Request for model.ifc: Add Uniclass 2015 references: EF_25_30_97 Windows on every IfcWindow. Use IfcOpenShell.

First a look at what the model holds.

```python
import ifcopenshell

model = ifcopenshell.open("model.ifc")
print(model.schema)
print("classifications:", [c.Name for c in model.by_type("IfcClassification")])
for ifc_class in ("IfcDoor", "IfcRoof", "IfcStair", "IfcWall", "IfcWindow"):
    print(ifc_class, len(model.by_type(ifc_class)))
```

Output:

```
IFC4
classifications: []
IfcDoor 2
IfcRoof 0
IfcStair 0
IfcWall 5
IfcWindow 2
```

```python
import ifcopenshell
import ifcopenshell.api.classification

model = ifcopenshell.open("model.ifc")

system = ifcopenshell.api.classification.add_classification(model, classification="Uniclass 2015")

codes = {
    "IfcWindow": ("EF_25_30_97", "Windows"),
}
for ifc_class, (code, name) in codes.items():
    products = model.by_type(ifc_class)
    ifcopenshell.api.classification.add_reference(
        model, products=products, classification=system, identification=code, name=name
    )
    print(code, len(products))

model.write("model_edited.ifc")
```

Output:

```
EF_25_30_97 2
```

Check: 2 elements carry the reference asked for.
